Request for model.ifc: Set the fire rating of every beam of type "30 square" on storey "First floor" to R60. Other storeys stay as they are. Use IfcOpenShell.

First a look at what the model holds.

```python
import ifcopenshell
import ifcopenshell.util.element

model = ifcopenshell.open("model.ifc")
print(model.schema)
storey = next(s for s in model.by_type("IfcBuildingStorey") if s.Name == "First floor")
beams = [e for e in ifcopenshell.util.element.get_decomposition(storey) if e.is_a("IfcBeam")]
seen = {}
for e in beams:
    element_type = ifcopenshell.util.element.get_type(e)
    key = (element_type.Name if element_type != e and element_type else None, ifcopenshell.util.element.get_pset(e, "Pset_BeamCommon", "FireRating"))
    seen[key] = seen.get(key, 0) + 1
for (name, value), count in sorted(seen.items(), key=str):
    print(count, "x", name, "|", value)
```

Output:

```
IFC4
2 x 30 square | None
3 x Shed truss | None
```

```python
import ifcopenshell
import ifcopenshell.api.pset
import ifcopenshell.util.element

model = ifcopenshell.open("model.ifc")

storey = next(s for s in model.by_type("IfcBuildingStorey") if s.Name == "First floor")
beams = [e for e in ifcopenshell.util.element.get_decomposition(storey) if e.is_a("IfcBeam")]

count = 0
for e in beams:
    element_type = ifcopenshell.util.element.get_type(e)
    if element_type in (None, e) or element_type.Name != "30 square":
        continue
    # add_pset returns the element's existing set when there is one.
    pset = ifcopenshell.api.pset.add_pset(model, product=e, name="Pset_BeamCommon")
    ifcopenshell.api.pset.edit_pset(model, pset=pset, properties={"FireRating": "R60"})
    count += 1

print(count, "beams updated")

model.write("model_rev.ifc")
```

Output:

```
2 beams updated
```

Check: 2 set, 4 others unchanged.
